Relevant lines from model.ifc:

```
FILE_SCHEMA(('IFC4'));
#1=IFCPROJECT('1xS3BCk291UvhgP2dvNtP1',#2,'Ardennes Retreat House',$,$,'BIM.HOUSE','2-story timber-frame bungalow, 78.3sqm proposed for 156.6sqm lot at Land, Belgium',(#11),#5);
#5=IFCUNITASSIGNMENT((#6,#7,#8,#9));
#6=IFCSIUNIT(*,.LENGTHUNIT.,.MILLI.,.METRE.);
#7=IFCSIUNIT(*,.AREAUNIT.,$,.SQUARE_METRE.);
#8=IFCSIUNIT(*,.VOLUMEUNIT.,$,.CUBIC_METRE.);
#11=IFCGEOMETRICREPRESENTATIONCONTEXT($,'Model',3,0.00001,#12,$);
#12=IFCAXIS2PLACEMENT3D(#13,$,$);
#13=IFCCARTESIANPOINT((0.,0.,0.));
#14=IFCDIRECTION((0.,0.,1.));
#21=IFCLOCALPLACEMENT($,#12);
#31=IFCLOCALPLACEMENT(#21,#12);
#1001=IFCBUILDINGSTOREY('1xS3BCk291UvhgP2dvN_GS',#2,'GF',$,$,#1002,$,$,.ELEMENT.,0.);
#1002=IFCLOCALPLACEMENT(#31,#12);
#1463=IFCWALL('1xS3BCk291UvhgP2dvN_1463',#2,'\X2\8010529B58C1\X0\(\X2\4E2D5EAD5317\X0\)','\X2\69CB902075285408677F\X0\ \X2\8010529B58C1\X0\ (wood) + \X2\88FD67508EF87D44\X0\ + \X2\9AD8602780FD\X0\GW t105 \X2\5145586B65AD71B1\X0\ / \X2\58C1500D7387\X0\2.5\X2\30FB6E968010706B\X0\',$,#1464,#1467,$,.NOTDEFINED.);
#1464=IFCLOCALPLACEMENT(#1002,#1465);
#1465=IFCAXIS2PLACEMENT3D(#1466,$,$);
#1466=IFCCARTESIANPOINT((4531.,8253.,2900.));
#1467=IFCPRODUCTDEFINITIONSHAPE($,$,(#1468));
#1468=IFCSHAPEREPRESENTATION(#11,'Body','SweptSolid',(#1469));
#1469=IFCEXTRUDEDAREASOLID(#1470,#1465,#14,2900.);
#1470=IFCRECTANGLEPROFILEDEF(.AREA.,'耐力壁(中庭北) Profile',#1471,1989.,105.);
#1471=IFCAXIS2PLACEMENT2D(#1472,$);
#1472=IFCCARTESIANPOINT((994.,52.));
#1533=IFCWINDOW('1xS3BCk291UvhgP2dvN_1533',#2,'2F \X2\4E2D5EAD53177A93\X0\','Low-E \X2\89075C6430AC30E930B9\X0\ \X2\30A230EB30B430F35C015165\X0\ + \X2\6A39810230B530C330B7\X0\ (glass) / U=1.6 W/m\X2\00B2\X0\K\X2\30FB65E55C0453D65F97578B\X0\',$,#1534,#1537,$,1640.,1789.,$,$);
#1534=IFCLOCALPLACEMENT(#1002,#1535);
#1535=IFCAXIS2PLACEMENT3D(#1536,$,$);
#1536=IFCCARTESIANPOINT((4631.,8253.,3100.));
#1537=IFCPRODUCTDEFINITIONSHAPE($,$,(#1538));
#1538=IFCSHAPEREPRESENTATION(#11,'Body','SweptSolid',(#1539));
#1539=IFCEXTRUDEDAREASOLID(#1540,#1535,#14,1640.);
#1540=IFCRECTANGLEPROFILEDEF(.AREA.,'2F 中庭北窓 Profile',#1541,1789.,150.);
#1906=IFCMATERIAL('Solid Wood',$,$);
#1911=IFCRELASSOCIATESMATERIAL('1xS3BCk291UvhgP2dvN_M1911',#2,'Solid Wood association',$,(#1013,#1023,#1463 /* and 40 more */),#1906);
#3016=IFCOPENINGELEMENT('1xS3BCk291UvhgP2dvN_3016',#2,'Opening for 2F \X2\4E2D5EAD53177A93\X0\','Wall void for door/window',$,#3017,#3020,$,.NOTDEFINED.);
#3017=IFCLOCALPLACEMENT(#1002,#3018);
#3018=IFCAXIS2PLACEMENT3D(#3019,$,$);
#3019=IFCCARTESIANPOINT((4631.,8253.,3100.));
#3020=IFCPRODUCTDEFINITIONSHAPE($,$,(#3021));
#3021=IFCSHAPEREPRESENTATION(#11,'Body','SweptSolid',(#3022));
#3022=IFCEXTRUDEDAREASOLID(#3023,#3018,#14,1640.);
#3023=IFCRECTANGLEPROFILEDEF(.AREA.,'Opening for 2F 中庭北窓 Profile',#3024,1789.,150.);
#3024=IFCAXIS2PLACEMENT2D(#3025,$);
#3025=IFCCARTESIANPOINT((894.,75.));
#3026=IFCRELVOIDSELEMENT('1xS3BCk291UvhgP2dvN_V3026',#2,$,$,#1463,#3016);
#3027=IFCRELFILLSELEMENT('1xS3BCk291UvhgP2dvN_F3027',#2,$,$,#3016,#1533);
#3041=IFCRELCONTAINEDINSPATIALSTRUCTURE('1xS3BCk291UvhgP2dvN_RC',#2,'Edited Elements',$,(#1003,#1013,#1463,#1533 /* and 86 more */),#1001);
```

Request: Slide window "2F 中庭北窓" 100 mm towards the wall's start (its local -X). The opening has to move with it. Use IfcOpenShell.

```python
import ifcopenshell
import ifcopenshell.api.geometry
import ifcopenshell.util.placement

model = ifcopenshell.open("model.ifc")

window = model.by_guid("1xS3BCk291UvhgP2dvN_1533")
opening = window.FillsVoids[0].RelatingOpeningElement
wall = opening.VoidsElements[0].RelatingBuildingElement

wall_matrix = ifcopenshell.util.placement.get_local_placement(wall.ObjectPlacement)
shift = wall_matrix[:3, 0] * -100.0
before = ifcopenshell.util.placement.get_local_placement(window.ObjectPlacement)[:3, 3].copy()

# The window is not placed relative to its opening, so move both.
for product in (opening, window):
    matrix = ifcopenshell.util.placement.get_local_placement(product.ObjectPlacement)
    matrix[:3, 3] += shift
    ifcopenshell.api.geometry.edit_object_placement(model, product=product, matrix=matrix, is_si=False)

after = ifcopenshell.util.placement.get_local_placement(window.ObjectPlacement)[:3, 3]
print("window moved by", (after - before).round(3) + 0.0)

model.write("model_updated.ifc")
```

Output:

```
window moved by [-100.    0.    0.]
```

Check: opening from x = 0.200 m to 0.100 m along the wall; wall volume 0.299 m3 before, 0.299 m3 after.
